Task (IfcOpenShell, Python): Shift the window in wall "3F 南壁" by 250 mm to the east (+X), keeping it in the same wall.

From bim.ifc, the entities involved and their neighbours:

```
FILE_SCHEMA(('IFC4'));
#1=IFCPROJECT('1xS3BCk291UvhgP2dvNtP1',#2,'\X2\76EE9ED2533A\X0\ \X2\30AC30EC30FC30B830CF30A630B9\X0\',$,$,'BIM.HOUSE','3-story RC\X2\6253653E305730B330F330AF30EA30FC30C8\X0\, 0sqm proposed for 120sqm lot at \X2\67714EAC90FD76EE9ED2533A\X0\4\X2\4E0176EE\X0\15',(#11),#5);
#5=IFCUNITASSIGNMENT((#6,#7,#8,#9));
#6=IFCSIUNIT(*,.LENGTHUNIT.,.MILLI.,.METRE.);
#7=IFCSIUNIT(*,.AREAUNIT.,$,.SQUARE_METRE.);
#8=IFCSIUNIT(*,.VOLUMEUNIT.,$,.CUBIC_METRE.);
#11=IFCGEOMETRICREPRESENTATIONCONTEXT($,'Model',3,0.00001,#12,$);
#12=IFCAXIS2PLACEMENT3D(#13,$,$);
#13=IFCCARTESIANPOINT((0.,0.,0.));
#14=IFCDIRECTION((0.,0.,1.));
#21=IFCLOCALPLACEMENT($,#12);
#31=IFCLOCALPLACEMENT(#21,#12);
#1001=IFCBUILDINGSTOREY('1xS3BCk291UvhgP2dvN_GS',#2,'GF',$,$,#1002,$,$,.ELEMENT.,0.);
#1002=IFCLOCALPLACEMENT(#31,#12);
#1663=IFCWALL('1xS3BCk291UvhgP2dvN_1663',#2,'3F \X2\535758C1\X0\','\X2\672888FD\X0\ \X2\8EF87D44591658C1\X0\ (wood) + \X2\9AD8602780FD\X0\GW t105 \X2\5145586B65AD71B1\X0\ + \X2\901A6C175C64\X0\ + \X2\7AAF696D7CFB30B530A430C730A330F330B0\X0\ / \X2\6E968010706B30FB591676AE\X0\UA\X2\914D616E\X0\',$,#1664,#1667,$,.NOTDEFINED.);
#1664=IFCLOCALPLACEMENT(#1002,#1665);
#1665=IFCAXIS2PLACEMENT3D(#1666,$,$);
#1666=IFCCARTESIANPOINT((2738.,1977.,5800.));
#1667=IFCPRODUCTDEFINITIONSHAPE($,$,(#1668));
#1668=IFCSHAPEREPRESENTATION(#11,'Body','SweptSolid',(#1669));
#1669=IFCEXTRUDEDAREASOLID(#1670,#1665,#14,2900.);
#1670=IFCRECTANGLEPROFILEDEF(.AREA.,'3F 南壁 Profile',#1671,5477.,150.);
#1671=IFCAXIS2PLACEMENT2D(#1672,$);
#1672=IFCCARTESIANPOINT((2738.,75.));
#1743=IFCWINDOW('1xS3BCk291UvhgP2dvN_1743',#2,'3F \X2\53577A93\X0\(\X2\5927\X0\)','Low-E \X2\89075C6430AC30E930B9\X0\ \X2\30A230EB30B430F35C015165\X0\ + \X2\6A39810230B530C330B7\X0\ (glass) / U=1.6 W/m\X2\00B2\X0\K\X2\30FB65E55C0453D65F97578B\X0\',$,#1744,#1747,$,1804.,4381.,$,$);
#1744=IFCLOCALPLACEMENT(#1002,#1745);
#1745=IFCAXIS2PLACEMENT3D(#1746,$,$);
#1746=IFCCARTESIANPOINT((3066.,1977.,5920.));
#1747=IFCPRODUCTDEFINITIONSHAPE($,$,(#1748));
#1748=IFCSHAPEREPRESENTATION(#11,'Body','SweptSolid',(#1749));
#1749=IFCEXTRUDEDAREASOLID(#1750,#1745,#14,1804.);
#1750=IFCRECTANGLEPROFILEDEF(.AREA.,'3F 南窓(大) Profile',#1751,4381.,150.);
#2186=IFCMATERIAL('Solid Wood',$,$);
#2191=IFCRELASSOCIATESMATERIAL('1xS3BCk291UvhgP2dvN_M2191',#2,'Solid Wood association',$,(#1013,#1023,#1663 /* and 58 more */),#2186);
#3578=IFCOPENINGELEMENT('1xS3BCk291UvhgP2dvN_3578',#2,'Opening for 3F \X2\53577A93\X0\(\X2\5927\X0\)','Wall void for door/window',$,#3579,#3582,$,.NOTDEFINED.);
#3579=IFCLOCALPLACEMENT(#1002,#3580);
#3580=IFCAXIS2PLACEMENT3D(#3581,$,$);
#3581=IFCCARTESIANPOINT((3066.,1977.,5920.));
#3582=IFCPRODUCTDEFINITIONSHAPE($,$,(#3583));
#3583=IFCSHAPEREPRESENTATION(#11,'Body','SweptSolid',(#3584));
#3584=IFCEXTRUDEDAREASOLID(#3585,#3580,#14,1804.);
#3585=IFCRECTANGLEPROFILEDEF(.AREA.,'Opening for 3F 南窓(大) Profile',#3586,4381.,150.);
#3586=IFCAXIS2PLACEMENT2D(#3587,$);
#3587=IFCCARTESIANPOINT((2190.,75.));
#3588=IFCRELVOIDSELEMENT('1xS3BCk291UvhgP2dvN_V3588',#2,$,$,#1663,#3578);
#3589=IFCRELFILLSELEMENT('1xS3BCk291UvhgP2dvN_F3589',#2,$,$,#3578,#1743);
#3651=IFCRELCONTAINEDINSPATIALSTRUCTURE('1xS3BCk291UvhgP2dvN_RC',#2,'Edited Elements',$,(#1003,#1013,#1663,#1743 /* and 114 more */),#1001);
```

```python
import ifcopenshell
import ifcopenshell.api.geometry
import ifcopenshell.util.placement
import ifcopenshell.util.unit

model = ifcopenshell.open("bim.ifc")
unit_scale = ifcopenshell.util.unit.calculate_unit_scale(model)

window = model.by_guid("1xS3BCk291UvhgP2dvN_1743")
opening = window.FillsVoids[0].RelatingOpeningElement
wall = opening.VoidsElements[0].RelatingBuildingElement

wall_matrix = ifcopenshell.util.placement.get_local_placement(wall.ObjectPlacement)
shift = wall_matrix[:3, 0] * 0.25 / unit_scale
before = ifcopenshell.util.placement.get_local_placement(window.ObjectPlacement)[:3, 3].copy()

# The window is not placed relative to its opening, so move both.
for product in (opening, window):
    matrix = ifcopenshell.util.placement.get_local_placement(product.ObjectPlacement)
    matrix[:3, 3] += shift
    ifcopenshell.api.geometry.edit_object_placement(model, product=product, matrix=matrix, is_si=False)

after = ifcopenshell.util.placement.get_local_placement(window.ObjectPlacement)[:3, 3]
print("window moved by", (after - before).round(3) + 0.0)

model.write("bim-out.ifc")
```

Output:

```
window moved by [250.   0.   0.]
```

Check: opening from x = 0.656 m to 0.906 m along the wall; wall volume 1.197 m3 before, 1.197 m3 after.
